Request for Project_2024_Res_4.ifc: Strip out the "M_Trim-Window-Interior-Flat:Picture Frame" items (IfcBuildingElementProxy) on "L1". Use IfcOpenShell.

First a look at what the model holds.

```python
import ifcopenshell
import ifcopenshell.util.element

model = ifcopenshell.open("Project_2024_Res_4.ifc")
print(model.schema)
storey = next(s for s in model.by_type("IfcBuildingStorey") if s.Name == "L1")
proxies = [e for e in ifcopenshell.util.element.get_decomposition(storey) if e.is_a("IfcBuildingElementProxy")]
seen = {}
for e in proxies:
    element_type = ifcopenshell.util.element.get_type(e)
    name = element_type.Name if element_type not in (None, e) else None
    seen[name] = seen.get(name, 0) + 1
for name, count in sorted(seen.items(), key=str):
    print(count, "x", name)
```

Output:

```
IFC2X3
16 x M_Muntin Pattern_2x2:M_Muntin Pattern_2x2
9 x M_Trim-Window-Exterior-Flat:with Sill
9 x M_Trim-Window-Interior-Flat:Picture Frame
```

```python
import ifcopenshell
import ifcopenshell.api.root
import ifcopenshell.util.element

model = ifcopenshell.open("Project_2024_Res_4.ifc")

storey = next(s for s in model.by_type("IfcBuildingStorey") if s.Name == "L1")
proxies = [e for e in ifcopenshell.util.element.get_decomposition(storey) if e.is_a("IfcBuildingElementProxy")]
targets = [e for e in proxies if (t := ifcopenshell.util.element.get_type(e)) not in (None, e) and t.Name == "M_Trim-Window-Interior-Flat:Picture Frame"]

for e in targets:
    ifcopenshell.api.root.remove_product(model, product=e)
print(len(targets), "removed")

model.write("Project_2024_Res_4_v2.ifc")
```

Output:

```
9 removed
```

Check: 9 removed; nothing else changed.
